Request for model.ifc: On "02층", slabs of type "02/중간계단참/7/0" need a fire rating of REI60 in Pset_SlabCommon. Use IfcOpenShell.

First a look at what the model holds.

```python
import ifcopenshell
import ifcopenshell.util.element

model = ifcopenshell.open("model.ifc")
print(model.schema)
storey = next(s for s in model.by_type("IfcBuildingStorey") if s.Name == "02층")
slabs = [e for e in ifcopenshell.util.element.get_decomposition(storey) if e.is_a("IfcSlab")]
seen = {}
for e in slabs:
    element_type = ifcopenshell.util.element.get_type(e)
    key = (element_type.Name if element_type != e and element_type else None, ifcopenshell.util.element.get_pset(e, "Pset_SlabCommon", "FireRating"))
    seen[key] = seen.get(key, 0) + 1
for (name, value), count in sorted(seen.items(), key=str):
    print(count, "x", name, "|", value)
```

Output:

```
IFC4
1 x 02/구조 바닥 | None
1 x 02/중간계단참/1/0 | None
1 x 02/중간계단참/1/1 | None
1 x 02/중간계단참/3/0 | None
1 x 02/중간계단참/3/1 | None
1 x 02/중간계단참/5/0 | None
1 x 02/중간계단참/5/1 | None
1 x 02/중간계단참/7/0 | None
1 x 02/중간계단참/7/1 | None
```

```python
import ifcopenshell
import ifcopenshell.api.pset
import ifcopenshell.util.element

model = ifcopenshell.open("model.ifc")

storey = next(s for s in model.by_type("IfcBuildingStorey") if s.Name == "02층")
slabs = [e for e in ifcopenshell.util.element.get_decomposition(storey) if e.is_a("IfcSlab")]

count = 0
for e in slabs:
    element_type = ifcopenshell.util.element.get_type(e)
    if element_type in (None, e) or element_type.Name != "02/중간계단참/7/0":
        continue
    # add_pset returns the element's existing set when there is one.
    pset = ifcopenshell.api.pset.add_pset(model, product=e, name="Pset_SlabCommon")
    ifcopenshell.api.pset.edit_pset(model, pset=pset, properties={"FireRating": "REI60"})
    count += 1

print(count, "slabs updated")

model.write("model_updated.ifc")
```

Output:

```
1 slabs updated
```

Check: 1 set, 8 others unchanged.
